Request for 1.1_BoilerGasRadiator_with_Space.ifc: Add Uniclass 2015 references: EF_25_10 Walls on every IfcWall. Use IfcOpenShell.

First a look at what the model holds.

```python
import ifcopenshell

model = ifcopenshell.open("1.1_BoilerGasRadiator_with_Space.ifc")
print(model.schema)
print("classifications:", [c.Name for c in model.by_type("IfcClassification")])
for ifc_class in ("IfcDoor", "IfcRoof", "IfcStair", "IfcWall", "IfcWindow"):
    print(ifc_class, len(model.by_type(ifc_class)))
```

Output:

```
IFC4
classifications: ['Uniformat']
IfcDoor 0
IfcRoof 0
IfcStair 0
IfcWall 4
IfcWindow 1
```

```python
import ifcopenshell
import ifcopenshell.api.classification

model = ifcopenshell.open("1.1_BoilerGasRadiator_with_Space.ifc")

system = ifcopenshell.api.classification.add_classification(model, classification="Uniclass 2015")

codes = {
    "IfcWall": ("EF_25_10", "Walls"),
}
for ifc_class, (code, name) in codes.items():
    products = model.by_type(ifc_class)
    ifcopenshell.api.classification.add_reference(
        model, products=products, classification=system, identification=code, name=name
    )
    print(code, len(products))

model.write("1.1_BoilerGasRadiator_with_Space_v2.ifc")
```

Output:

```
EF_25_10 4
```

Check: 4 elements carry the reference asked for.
